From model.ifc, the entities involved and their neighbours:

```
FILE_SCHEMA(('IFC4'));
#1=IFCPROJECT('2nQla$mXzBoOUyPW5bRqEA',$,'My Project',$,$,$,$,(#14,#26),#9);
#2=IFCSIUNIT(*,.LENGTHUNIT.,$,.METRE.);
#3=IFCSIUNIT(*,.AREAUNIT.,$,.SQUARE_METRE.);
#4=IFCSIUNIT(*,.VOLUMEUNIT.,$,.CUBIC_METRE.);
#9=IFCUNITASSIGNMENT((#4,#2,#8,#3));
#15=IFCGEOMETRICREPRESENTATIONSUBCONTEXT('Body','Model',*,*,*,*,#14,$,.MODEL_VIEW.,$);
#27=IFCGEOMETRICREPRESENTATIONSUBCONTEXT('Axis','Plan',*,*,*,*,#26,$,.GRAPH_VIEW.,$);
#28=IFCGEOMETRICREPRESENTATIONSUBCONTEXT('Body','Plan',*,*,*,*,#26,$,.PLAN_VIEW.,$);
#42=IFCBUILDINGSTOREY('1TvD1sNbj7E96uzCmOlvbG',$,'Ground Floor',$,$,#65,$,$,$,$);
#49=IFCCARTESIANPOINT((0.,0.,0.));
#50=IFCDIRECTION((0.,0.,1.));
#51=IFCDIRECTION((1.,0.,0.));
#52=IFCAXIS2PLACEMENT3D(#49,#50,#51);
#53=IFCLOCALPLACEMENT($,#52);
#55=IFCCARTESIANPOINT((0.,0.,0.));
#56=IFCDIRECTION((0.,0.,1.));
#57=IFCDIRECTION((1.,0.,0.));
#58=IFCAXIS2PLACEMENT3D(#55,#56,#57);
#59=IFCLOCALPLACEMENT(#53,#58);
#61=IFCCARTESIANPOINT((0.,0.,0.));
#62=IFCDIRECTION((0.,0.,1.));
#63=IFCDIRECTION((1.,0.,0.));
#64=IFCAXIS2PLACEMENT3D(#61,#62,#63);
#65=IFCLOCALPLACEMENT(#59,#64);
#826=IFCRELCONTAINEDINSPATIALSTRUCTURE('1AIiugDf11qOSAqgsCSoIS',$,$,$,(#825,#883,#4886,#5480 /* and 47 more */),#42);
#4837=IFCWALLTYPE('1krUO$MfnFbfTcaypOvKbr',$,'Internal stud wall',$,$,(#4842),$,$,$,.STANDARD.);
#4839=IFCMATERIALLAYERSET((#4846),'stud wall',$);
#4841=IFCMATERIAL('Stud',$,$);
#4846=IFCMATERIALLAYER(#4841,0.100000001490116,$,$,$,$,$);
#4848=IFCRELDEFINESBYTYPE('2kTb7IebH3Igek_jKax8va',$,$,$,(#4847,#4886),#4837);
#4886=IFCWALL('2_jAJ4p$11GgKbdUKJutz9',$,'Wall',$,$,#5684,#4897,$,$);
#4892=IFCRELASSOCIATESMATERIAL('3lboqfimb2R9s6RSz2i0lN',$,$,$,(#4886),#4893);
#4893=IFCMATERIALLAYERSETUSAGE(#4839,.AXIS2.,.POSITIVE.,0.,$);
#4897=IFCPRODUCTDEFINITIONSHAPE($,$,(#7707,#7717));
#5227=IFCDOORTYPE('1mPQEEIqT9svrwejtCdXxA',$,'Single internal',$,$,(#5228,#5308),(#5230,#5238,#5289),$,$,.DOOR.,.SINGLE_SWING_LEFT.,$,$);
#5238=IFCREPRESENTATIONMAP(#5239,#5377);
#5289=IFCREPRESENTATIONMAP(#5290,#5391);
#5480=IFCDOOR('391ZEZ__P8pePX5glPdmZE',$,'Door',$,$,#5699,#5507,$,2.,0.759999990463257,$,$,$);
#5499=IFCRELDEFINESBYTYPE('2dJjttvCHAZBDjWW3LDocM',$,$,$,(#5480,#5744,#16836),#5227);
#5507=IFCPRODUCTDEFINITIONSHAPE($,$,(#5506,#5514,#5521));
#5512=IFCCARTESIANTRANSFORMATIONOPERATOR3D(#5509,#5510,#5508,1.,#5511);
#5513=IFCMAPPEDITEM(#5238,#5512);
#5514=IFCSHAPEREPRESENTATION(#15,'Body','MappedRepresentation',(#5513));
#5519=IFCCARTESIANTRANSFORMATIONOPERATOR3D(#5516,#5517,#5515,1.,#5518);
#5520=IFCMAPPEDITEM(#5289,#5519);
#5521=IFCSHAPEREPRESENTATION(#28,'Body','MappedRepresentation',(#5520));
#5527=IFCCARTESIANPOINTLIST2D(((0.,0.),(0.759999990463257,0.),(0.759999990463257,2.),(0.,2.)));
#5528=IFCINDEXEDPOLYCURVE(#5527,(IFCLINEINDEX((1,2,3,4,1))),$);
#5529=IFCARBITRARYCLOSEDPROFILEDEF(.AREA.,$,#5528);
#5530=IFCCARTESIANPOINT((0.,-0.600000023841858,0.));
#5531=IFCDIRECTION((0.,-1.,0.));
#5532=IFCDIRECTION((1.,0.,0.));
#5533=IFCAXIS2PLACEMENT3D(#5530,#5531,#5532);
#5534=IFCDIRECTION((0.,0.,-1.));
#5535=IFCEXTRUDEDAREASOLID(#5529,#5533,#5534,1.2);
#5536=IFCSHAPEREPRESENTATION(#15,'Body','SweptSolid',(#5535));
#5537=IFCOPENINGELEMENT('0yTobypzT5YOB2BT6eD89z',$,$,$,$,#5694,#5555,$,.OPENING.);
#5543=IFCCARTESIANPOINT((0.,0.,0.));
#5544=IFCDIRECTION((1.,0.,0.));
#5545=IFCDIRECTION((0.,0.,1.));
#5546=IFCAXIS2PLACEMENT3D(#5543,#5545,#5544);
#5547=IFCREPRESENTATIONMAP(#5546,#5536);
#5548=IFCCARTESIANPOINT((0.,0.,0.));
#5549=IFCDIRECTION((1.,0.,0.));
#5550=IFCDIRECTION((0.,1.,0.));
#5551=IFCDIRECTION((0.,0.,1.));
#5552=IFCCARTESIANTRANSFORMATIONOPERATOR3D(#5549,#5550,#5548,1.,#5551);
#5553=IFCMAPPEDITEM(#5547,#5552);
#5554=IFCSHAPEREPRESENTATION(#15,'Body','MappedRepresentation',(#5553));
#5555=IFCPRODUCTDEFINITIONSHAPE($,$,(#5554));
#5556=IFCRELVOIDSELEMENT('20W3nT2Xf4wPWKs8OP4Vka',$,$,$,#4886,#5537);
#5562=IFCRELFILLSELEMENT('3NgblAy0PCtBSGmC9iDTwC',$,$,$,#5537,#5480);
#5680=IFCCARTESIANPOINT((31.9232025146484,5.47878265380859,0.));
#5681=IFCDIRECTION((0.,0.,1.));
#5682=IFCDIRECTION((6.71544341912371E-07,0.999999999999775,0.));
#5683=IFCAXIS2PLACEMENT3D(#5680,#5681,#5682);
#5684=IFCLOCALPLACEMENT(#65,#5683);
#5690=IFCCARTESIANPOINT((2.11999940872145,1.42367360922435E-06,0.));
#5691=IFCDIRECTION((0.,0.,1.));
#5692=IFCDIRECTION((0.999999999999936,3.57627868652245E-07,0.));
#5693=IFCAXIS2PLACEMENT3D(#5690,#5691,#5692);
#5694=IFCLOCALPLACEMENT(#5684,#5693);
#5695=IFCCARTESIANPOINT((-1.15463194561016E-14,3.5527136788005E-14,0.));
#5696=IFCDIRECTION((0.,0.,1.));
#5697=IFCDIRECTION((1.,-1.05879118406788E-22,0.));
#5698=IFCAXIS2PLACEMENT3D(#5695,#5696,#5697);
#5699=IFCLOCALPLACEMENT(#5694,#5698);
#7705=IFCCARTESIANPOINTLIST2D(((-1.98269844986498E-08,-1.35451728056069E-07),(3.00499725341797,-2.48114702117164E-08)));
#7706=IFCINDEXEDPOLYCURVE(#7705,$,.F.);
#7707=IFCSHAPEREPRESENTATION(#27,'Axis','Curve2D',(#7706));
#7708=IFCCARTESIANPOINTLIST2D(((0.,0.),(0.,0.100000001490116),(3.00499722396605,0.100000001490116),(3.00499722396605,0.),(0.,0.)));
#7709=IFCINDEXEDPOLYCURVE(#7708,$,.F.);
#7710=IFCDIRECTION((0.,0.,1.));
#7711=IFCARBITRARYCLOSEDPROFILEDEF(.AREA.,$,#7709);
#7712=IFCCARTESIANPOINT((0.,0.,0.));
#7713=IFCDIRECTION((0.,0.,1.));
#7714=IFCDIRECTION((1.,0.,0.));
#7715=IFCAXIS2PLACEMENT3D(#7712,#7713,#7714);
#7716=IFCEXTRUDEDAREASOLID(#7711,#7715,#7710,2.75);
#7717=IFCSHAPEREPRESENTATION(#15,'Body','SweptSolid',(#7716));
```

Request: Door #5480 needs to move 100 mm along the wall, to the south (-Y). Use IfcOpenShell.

```python
import ifcopenshell
import ifcopenshell.api.geometry
import ifcopenshell.util.placement

model = ifcopenshell.open("model.ifc")

door = model.by_guid("391ZEZ__P8pePX5glPdmZE")
opening = door.FillsVoids[0].RelatingOpeningElement
wall = opening.VoidsElements[0].RelatingBuildingElement

wall_matrix = ifcopenshell.util.placement.get_local_placement(wall.ObjectPlacement)
shift = wall_matrix[:3, 0] * -0.1
before = ifcopenshell.util.placement.get_local_placement(door.ObjectPlacement)[:3, 3].copy()

# The door is placed relative to its opening, so it follows when the opening moves.
matrix = ifcopenshell.util.placement.get_local_placement(opening.ObjectPlacement)
matrix[:3, 3] += shift
ifcopenshell.api.geometry.edit_object_placement(
    model, product=opening, matrix=matrix, is_si=False, should_transform_children=True
)

after = ifcopenshell.util.placement.get_local_placement(door.ObjectPlacement)[:3, 3]
print("door moved by", (after - before).round(3) + 0.0)

model.write("model_updated.ifc")
```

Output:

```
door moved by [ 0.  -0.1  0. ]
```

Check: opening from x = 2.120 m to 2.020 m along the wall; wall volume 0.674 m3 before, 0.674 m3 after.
